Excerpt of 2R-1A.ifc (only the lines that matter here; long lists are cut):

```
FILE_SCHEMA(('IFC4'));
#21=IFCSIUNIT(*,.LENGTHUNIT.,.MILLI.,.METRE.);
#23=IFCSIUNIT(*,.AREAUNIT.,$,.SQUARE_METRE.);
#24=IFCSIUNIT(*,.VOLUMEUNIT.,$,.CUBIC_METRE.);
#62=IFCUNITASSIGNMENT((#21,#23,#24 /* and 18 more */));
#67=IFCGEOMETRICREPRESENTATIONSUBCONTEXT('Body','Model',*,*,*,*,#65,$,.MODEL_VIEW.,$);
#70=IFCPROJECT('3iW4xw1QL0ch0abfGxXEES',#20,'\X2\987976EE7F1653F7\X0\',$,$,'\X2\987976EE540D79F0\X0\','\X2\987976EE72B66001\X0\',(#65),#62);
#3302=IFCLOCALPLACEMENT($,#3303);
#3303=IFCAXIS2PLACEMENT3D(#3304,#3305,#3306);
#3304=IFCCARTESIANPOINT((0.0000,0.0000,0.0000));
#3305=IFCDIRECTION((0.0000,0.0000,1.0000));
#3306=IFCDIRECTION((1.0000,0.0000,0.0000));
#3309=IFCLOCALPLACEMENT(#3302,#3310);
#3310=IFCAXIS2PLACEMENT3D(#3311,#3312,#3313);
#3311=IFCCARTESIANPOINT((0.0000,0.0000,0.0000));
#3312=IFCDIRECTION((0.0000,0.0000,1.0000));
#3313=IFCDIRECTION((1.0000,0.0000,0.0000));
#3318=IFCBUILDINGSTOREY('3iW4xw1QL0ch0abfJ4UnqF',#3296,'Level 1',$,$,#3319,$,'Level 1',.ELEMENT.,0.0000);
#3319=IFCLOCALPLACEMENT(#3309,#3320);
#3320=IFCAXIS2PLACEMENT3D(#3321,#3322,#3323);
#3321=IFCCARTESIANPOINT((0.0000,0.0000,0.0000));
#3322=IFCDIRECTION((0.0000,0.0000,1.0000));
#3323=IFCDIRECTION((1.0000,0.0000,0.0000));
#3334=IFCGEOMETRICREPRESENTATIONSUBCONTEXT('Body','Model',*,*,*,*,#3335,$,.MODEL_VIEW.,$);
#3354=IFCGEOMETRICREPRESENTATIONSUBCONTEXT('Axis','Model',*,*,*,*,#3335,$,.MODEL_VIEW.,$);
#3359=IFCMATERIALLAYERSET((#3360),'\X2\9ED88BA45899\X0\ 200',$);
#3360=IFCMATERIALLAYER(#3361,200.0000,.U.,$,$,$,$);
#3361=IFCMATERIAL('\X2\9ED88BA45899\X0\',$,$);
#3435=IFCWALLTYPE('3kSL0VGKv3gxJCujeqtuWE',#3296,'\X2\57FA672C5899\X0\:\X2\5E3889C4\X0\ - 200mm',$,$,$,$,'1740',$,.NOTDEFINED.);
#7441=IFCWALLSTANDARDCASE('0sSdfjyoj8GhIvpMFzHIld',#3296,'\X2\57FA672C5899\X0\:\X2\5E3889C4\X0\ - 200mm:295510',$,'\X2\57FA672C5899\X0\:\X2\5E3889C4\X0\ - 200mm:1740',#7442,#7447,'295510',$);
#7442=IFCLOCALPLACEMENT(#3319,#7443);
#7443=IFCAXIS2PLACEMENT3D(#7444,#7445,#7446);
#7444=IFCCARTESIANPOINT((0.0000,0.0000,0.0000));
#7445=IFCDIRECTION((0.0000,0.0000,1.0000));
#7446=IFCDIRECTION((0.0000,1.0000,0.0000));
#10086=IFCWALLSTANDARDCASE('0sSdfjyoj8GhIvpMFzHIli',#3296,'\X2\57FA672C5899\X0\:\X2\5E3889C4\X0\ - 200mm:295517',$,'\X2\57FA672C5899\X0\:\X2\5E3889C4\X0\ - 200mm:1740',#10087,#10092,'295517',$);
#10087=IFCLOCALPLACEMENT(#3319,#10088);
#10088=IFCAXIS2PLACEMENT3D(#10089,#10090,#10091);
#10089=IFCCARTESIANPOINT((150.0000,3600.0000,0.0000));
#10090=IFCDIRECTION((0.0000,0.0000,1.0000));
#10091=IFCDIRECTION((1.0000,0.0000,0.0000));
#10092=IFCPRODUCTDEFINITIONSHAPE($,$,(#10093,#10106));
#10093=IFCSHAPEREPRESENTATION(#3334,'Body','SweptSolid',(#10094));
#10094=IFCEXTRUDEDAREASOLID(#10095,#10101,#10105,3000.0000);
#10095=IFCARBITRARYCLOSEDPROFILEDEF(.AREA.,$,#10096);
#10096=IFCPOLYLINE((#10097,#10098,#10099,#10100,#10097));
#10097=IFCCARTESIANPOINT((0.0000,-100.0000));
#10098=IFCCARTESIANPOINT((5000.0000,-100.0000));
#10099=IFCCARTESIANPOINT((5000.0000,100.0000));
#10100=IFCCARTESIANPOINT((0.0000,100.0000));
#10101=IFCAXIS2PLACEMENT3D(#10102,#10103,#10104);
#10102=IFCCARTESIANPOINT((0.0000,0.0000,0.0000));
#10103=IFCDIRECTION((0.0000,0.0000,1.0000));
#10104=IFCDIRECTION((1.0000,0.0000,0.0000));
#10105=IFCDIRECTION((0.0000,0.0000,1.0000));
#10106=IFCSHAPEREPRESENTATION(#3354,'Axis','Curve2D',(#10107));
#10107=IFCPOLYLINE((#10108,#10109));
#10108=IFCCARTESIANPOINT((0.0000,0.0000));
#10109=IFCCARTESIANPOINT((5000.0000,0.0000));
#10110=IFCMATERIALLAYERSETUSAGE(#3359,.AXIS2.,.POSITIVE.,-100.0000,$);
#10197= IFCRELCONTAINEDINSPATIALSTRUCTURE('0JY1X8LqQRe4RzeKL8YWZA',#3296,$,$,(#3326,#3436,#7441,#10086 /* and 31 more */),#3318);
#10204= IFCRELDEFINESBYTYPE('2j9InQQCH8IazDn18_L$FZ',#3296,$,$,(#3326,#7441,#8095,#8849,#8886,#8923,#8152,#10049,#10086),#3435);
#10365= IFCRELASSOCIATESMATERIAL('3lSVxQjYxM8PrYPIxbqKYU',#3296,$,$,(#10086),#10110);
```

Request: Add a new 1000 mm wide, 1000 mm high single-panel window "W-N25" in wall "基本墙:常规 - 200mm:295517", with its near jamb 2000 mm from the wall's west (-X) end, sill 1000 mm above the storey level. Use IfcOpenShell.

```python
import numpy as np
import ifcopenshell
import ifcopenshell.api.feature
import ifcopenshell.api.geometry
import ifcopenshell.api.root
import ifcopenshell.api.spatial
import ifcopenshell.geom
import ifcopenshell.util.element
import ifcopenshell.util.placement
import ifcopenshell.util.representation
import ifcopenshell.util.shape
import ifcopenshell.util.unit

model = ifcopenshell.open("2R-1A.ifc")
unit_scale = ifcopenshell.util.unit.calculate_unit_scale(model)
settings = ifcopenshell.geom.settings()


def volume(element):
    """Net volume in cubic metres, openings subtracted."""
    shape = ifcopenshell.geom.create_shape(settings, element)
    return ifcopenshell.util.shape.get_volume(shape.geometry)


wall = model.by_guid("0sSdfjyoj8GhIvpMFzHIli")
storey = ifcopenshell.util.element.get_container(wall, ifc_class="IfcBuildingStorey")
context = ifcopenshell.util.representation.get_context(model, "Model", "Body", "MODEL_VIEW")
before = volume(wall)

width, height, from_end, sill = 1, 1, 2, 1  # metres

# The wall runs along its own X axis, and the end named is its -X end.
wall_shape = ifcopenshell.geom.create_shape(settings, wall)
x, y, z = ifcopenshell.util.shape.get_vertices(wall_shape.geometry).T
start = x.min() + from_end
face, thickness = float(y.min()), float(y.max() - y.min())
wall_matrix = ifcopenshell.util.placement.get_local_placement(wall.ObjectPlacement)
level = ifcopenshell.util.placement.get_local_placement(storey.ObjectPlacement)[2, 3]


def in_wall(x, y):
    """Placement at x, y metres in the wall's axes, at sill height."""
    matrix = wall_matrix.copy()
    matrix[:, 3] = wall_matrix @ np.array([x / unit_scale, y / unit_scale, 0.0, 1.0])
    matrix[2, 3] = level + sill / unit_scale
    return matrix


# Opening: a box that overshoots both wall faces by 50 mm.
opening = ifcopenshell.api.root.create_entity(model, ifc_class="IfcOpeningElement", predefined_type="OPENING")
box = ifcopenshell.api.geometry.add_wall_representation(
    model, context=context, length=width, height=height, thickness=thickness + 0.1
)
ifcopenshell.api.geometry.assign_representation(model, product=opening, representation=box)
ifcopenshell.api.geometry.edit_object_placement(model, product=opening, matrix=in_wall(start, face - 0.05), is_si=False)
ifcopenshell.api.feature.add_feature(model, feature=opening, element=wall)

window = ifcopenshell.api.root.create_entity(model, ifc_class="IfcWindow", name="W-N25", predefined_type="WINDOW")
window.OverallWidth, window.OverallHeight = width / unit_scale, height / unit_scale
window.PartitioningType = "SINGLE_PANEL"
body = ifcopenshell.api.geometry.add_window_representation(
    model,
    context=context,
    overall_width=window.OverallWidth,
    overall_height=window.OverallHeight,
    partition_type="SINGLE_PANEL",
)
ifcopenshell.api.geometry.assign_representation(model, product=window, representation=body)
ifcopenshell.api.spatial.assign_container(model, products=[window], relating_structure=storey)
ifcopenshell.api.feature.add_filling(model, opening=opening, element=window)

# Centre the window in the wall's thickness.
ifcopenshell.api.geometry.edit_object_placement(model, product=window, matrix=in_wall(start, face), is_si=False)
window_shape = ifcopenshell.geom.create_shape(settings, window)
depth = ifcopenshell.util.shape.get_vertices(window_shape.geometry)[:, 1]
offset = face + thickness / 2 - (depth.min() + depth.max()) / 2
ifcopenshell.api.geometry.edit_object_placement(model, product=window, matrix=in_wall(start, offset), is_si=False)

after = volume(wall)

print(f"wall volume {before:.3f} -> {after:.3f} m3")

model.write("2R-1A-out.ifc")
```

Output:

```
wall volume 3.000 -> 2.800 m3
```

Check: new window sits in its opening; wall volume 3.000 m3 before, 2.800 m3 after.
